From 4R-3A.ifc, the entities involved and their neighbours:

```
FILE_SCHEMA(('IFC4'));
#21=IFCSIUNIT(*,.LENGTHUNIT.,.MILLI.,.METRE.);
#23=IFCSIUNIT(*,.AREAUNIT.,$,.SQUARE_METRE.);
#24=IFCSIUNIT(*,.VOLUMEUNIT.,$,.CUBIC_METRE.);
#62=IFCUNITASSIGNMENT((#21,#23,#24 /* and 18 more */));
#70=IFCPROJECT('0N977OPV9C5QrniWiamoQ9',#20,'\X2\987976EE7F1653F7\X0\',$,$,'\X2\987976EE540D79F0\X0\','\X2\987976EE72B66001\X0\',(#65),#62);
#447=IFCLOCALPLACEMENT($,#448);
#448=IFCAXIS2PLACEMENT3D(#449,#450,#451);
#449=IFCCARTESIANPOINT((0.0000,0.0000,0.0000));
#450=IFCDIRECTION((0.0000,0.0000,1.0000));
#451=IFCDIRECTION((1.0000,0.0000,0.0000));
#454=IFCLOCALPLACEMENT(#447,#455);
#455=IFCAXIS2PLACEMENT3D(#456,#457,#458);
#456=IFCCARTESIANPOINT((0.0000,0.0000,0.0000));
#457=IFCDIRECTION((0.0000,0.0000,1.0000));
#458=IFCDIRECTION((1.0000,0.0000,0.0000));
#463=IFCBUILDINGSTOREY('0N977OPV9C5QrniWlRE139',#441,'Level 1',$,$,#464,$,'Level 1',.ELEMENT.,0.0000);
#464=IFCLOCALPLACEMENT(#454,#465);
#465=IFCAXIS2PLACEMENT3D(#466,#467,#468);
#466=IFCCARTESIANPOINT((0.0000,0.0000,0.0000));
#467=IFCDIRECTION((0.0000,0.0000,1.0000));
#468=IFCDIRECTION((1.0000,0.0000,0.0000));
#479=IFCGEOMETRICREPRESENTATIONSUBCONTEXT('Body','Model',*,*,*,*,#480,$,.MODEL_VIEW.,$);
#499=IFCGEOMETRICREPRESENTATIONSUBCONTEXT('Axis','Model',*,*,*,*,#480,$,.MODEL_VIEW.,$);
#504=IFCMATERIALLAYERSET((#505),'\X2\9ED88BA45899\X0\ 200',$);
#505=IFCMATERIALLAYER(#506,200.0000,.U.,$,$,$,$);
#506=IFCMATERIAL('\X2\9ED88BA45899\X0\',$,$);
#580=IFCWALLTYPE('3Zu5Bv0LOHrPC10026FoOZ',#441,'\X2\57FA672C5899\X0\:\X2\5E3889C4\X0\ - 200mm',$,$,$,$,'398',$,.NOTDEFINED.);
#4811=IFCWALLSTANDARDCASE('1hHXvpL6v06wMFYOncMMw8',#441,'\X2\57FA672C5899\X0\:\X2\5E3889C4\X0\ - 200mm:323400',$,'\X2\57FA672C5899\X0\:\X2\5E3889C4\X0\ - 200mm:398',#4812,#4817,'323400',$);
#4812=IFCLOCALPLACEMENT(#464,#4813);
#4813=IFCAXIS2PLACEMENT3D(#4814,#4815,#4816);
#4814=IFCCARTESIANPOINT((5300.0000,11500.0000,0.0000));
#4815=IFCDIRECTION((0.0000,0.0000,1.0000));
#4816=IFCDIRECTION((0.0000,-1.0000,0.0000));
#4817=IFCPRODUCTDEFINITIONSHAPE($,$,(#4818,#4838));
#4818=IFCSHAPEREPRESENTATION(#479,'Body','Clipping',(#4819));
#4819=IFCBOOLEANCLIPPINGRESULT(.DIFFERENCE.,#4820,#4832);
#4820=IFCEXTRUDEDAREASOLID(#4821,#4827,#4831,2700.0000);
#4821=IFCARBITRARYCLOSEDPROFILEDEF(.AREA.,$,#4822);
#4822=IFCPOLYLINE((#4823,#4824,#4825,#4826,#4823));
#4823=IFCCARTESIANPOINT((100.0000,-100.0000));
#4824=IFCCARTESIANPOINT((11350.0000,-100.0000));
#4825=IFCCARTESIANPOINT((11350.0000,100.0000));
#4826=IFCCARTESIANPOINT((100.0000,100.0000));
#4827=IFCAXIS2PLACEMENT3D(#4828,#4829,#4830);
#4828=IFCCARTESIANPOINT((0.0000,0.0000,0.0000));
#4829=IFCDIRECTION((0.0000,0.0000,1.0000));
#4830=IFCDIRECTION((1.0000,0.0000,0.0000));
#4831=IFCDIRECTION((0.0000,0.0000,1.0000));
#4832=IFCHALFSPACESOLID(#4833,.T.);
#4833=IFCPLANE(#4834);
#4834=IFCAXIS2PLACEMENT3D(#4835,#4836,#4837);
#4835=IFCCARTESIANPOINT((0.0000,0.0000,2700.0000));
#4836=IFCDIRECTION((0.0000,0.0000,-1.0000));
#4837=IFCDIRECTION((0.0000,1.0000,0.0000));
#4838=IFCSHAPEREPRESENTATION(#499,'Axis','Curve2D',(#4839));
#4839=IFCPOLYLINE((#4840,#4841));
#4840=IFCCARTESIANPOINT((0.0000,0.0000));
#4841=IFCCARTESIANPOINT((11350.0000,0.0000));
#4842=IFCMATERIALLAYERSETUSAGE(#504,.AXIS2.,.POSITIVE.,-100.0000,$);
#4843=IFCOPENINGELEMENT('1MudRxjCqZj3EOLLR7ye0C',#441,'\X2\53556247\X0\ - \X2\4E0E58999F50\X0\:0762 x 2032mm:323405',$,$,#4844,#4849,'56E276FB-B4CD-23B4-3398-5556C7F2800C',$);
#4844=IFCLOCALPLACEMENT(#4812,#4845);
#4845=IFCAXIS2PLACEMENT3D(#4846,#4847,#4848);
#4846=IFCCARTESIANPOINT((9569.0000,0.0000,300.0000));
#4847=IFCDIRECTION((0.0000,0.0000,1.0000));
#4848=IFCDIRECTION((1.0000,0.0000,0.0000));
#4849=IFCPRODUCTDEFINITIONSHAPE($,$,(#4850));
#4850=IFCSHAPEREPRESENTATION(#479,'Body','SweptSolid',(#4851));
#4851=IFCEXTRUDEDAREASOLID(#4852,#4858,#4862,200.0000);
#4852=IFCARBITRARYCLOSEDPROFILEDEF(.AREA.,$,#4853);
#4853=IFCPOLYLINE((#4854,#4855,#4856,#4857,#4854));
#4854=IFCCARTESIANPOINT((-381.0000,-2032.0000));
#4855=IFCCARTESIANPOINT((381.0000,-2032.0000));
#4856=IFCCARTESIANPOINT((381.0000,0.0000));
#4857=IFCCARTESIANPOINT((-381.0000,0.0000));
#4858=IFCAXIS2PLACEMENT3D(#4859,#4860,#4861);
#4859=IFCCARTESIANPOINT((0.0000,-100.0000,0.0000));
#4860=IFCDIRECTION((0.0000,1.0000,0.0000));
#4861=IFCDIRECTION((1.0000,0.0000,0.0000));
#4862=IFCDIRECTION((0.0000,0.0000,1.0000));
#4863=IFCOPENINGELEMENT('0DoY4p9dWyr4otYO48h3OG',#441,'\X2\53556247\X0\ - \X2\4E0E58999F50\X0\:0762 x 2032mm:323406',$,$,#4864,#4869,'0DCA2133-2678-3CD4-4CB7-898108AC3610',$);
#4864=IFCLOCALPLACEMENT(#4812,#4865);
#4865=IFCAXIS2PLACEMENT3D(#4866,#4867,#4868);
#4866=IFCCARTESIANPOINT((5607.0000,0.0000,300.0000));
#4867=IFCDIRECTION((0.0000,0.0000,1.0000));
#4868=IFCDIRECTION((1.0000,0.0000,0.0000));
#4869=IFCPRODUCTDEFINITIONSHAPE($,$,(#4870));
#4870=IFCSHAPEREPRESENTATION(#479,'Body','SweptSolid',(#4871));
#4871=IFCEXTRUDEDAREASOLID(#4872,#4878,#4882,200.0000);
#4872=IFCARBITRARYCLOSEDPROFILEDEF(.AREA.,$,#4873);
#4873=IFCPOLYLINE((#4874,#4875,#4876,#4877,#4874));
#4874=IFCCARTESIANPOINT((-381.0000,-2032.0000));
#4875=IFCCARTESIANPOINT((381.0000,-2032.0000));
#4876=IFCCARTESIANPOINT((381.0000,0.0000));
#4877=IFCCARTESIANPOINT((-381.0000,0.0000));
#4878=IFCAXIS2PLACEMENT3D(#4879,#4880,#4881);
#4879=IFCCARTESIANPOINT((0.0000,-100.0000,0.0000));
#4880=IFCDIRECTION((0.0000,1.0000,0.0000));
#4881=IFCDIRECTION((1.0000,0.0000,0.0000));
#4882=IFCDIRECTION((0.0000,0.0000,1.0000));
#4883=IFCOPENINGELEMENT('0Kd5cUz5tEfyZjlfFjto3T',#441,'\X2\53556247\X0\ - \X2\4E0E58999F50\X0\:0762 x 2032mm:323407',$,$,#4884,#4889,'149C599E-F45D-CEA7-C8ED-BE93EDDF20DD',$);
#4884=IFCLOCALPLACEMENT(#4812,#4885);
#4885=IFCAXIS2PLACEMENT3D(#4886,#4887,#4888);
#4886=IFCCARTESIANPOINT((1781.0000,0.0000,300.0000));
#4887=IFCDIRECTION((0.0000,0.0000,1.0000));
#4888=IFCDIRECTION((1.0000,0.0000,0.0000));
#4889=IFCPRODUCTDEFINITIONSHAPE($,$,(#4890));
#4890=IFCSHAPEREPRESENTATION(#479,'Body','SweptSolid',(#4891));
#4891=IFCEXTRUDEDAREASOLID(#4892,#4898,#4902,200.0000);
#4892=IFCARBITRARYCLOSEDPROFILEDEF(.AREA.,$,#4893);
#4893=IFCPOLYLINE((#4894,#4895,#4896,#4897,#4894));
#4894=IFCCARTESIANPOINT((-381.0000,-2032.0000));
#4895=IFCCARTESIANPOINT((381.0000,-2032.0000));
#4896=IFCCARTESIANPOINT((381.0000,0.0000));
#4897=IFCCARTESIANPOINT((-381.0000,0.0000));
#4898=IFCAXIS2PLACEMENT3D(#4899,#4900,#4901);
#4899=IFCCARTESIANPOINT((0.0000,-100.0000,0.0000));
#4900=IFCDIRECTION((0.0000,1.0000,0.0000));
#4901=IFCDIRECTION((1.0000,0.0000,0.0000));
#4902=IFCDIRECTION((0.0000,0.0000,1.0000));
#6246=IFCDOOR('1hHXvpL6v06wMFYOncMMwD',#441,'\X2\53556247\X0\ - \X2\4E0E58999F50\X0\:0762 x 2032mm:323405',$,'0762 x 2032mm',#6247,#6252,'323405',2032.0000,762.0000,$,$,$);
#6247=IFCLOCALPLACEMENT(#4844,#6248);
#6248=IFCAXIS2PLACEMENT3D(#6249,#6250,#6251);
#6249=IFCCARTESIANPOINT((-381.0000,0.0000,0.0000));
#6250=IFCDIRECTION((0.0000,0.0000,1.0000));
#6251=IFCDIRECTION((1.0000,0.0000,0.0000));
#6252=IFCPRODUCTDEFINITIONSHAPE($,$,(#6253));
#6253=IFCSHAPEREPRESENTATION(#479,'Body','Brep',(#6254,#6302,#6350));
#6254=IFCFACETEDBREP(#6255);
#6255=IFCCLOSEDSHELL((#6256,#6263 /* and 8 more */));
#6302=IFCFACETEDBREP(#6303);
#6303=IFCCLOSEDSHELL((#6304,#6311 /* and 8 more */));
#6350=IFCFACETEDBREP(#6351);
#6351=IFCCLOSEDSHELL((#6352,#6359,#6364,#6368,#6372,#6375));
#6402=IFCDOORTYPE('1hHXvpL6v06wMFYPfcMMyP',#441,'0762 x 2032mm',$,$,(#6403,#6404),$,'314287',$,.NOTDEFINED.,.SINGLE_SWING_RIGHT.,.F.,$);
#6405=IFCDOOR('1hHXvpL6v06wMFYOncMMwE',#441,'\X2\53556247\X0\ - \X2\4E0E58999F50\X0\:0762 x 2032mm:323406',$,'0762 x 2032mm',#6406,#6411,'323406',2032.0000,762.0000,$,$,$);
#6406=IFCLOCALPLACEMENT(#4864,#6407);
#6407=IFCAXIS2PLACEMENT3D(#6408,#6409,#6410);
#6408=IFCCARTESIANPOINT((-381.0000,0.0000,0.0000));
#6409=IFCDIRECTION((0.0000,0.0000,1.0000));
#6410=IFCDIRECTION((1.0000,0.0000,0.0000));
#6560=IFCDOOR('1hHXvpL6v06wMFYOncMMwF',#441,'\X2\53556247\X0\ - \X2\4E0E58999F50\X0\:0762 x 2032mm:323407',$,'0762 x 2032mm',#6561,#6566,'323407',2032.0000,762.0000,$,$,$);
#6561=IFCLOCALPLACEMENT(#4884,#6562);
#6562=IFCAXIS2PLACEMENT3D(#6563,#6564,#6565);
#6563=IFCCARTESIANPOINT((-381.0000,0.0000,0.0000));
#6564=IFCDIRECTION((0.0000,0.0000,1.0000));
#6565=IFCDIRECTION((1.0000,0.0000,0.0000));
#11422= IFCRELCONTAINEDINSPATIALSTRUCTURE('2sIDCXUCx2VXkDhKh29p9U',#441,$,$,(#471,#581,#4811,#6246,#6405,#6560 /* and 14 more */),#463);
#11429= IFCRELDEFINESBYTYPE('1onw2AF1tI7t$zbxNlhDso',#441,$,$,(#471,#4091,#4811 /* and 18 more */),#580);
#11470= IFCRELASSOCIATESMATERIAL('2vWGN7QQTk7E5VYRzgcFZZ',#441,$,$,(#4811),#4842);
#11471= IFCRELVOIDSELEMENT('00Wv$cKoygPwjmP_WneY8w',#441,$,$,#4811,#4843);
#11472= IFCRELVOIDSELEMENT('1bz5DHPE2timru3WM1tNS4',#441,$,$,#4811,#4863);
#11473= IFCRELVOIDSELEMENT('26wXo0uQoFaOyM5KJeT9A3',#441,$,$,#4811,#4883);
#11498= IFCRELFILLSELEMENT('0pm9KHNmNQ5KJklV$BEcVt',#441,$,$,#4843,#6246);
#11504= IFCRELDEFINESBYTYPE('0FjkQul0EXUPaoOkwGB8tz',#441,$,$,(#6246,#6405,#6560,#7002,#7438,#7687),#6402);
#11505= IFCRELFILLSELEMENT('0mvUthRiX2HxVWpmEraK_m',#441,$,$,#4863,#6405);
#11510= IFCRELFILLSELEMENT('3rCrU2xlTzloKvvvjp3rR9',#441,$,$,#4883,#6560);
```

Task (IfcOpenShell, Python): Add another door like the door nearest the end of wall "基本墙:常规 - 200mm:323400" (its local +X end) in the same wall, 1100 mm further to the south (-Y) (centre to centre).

```python
import ifcopenshell
import ifcopenshell.api.feature
import ifcopenshell.api.geometry
import ifcopenshell.api.root
import ifcopenshell.geom
import ifcopenshell.util.element
import ifcopenshell.util.placement
import ifcopenshell.util.shape

model = ifcopenshell.open("4R-3A.ifc")
settings = ifcopenshell.geom.settings()


def volume(element):
    """Net volume in cubic metres, openings subtracted."""
    shape = ifcopenshell.geom.create_shape(settings, element)
    return ifcopenshell.util.shape.get_volume(shape.geometry)


def reuse_history(source, copy):
    """copy_class also copies each property set's owner history, people and application; keep the originals."""
    for rel in copy.IsDefinedBy:
        if rel.is_a("IfcRelDefinesByProperties") and (history := rel.RelatingPropertyDefinition.OwnerHistory):
            rel.RelatingPropertyDefinition.OwnerHistory = source.OwnerHistory
            ifcopenshell.util.element.remove_deep2(model, history)


door = model.by_id(6246)
opening = door.FillsVoids[0].RelatingOpeningElement
wall = opening.VoidsElements[0].RelatingBuildingElement
before = volume(wall)
shift = ifcopenshell.util.placement.get_local_placement(wall.ObjectPlacement)[:3, 0] * 1100.0

# copy_class copies the void relationship, type, container and properties, but no geometry.
new_opening = ifcopenshell.api.root.copy_class(model, product=opening)
new_opening.Representation = ifcopenshell.util.element.copy_deep(
    model, opening.Representation, exclude=["IfcGeometricRepresentationContext", "IfcRepresentationMap"]
)
new_opening.Name = "单扇 - 与墙齐:0762 x 2032mm"
new_opening.Tag = None
new_door = ifcopenshell.api.root.copy_class(model, product=door)
new_door.Representation = ifcopenshell.util.element.copy_deep(
    model, door.Representation, exclude=["IfcGeometricRepresentationContext", "IfcRepresentationMap"]
)
new_door.Name = "单扇 - 与墙齐:0762 x 2032mm"
new_door.Tag = None
reuse_history(door, new_door)
ifcopenshell.api.feature.add_filling(model, opening=new_opening, element=new_door)

for old, new in ((opening, new_opening), (door, new_door)):
    matrix = ifcopenshell.util.placement.get_local_placement(old.ObjectPlacement)
    matrix[:3, 3] += shift
    ifcopenshell.api.geometry.edit_object_placement(model, product=new, matrix=matrix, is_si=False)

after = volume(wall)

print(f"wall volume {before:.3f} -> {after:.3f} m3")

model.write("4R-3A_rev.ifc")
```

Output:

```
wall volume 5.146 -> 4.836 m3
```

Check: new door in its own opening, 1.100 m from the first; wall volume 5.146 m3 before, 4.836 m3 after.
